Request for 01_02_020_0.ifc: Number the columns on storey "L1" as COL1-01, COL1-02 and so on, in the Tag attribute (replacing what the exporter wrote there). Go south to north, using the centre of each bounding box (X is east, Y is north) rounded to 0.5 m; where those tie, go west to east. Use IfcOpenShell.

First a look at what the model holds.

```python
import ifcopenshell
import ifcopenshell.util.element
import ifcopenshell.util.placement

model = ifcopenshell.open("01_02_020_0.ifc")
print(model.schema)
storey = next(s for s in model.by_type("IfcBuildingStorey") if s.Name == "L1")
columns = [e for e in ifcopenshell.util.element.get_decomposition(storey) if e.is_a("IfcColumn")]
for e in sorted(columns, key=lambda e: e.id()):
    origin = ifcopenshell.util.placement.get_local_placement(e.ObjectPlacement)[:3, 3]
    print(e.id(), e.Tag, e.Name, origin.round(2) + 0.0, sep=" | ")
```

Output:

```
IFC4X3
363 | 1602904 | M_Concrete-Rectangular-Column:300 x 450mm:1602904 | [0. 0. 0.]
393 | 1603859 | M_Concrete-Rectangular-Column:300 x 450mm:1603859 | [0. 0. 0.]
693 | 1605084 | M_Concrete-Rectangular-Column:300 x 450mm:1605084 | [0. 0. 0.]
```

```python
import ifcopenshell
import ifcopenshell.geom
import ifcopenshell.util.element
import ifcopenshell.util.shape

model = ifcopenshell.open("01_02_020_0.ifc")
settings = ifcopenshell.geom.settings()
settings.set("use-world-coords", True)


def centre(element):
    shape = ifcopenshell.geom.create_shape(settings, element)
    return ifcopenshell.util.shape.get_bbox_centroid(shape.geometry)


storey = next(s for s in model.by_type("IfcBuildingStorey") if s.Name == "L1")
columns = [e for e in ifcopenshell.util.element.get_decomposition(storey) if e.is_a("IfcColumn")]

# Insertion points can sit at a corner or the storey origin, so sort by the geometry (in metres).
centres = {e: centre(e) for e in columns}
columns.sort(key=lambda e: (round(centres[e][1] / 0.5), centres[e][0]))

for i, e in enumerate(columns, start=1):
    number = f"COL1-{i:02d}"
    e.Tag = number
    print(e.id(), number)

model.write("01_02_020_0_v2.ifc")
```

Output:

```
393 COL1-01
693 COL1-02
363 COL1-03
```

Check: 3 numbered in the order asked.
